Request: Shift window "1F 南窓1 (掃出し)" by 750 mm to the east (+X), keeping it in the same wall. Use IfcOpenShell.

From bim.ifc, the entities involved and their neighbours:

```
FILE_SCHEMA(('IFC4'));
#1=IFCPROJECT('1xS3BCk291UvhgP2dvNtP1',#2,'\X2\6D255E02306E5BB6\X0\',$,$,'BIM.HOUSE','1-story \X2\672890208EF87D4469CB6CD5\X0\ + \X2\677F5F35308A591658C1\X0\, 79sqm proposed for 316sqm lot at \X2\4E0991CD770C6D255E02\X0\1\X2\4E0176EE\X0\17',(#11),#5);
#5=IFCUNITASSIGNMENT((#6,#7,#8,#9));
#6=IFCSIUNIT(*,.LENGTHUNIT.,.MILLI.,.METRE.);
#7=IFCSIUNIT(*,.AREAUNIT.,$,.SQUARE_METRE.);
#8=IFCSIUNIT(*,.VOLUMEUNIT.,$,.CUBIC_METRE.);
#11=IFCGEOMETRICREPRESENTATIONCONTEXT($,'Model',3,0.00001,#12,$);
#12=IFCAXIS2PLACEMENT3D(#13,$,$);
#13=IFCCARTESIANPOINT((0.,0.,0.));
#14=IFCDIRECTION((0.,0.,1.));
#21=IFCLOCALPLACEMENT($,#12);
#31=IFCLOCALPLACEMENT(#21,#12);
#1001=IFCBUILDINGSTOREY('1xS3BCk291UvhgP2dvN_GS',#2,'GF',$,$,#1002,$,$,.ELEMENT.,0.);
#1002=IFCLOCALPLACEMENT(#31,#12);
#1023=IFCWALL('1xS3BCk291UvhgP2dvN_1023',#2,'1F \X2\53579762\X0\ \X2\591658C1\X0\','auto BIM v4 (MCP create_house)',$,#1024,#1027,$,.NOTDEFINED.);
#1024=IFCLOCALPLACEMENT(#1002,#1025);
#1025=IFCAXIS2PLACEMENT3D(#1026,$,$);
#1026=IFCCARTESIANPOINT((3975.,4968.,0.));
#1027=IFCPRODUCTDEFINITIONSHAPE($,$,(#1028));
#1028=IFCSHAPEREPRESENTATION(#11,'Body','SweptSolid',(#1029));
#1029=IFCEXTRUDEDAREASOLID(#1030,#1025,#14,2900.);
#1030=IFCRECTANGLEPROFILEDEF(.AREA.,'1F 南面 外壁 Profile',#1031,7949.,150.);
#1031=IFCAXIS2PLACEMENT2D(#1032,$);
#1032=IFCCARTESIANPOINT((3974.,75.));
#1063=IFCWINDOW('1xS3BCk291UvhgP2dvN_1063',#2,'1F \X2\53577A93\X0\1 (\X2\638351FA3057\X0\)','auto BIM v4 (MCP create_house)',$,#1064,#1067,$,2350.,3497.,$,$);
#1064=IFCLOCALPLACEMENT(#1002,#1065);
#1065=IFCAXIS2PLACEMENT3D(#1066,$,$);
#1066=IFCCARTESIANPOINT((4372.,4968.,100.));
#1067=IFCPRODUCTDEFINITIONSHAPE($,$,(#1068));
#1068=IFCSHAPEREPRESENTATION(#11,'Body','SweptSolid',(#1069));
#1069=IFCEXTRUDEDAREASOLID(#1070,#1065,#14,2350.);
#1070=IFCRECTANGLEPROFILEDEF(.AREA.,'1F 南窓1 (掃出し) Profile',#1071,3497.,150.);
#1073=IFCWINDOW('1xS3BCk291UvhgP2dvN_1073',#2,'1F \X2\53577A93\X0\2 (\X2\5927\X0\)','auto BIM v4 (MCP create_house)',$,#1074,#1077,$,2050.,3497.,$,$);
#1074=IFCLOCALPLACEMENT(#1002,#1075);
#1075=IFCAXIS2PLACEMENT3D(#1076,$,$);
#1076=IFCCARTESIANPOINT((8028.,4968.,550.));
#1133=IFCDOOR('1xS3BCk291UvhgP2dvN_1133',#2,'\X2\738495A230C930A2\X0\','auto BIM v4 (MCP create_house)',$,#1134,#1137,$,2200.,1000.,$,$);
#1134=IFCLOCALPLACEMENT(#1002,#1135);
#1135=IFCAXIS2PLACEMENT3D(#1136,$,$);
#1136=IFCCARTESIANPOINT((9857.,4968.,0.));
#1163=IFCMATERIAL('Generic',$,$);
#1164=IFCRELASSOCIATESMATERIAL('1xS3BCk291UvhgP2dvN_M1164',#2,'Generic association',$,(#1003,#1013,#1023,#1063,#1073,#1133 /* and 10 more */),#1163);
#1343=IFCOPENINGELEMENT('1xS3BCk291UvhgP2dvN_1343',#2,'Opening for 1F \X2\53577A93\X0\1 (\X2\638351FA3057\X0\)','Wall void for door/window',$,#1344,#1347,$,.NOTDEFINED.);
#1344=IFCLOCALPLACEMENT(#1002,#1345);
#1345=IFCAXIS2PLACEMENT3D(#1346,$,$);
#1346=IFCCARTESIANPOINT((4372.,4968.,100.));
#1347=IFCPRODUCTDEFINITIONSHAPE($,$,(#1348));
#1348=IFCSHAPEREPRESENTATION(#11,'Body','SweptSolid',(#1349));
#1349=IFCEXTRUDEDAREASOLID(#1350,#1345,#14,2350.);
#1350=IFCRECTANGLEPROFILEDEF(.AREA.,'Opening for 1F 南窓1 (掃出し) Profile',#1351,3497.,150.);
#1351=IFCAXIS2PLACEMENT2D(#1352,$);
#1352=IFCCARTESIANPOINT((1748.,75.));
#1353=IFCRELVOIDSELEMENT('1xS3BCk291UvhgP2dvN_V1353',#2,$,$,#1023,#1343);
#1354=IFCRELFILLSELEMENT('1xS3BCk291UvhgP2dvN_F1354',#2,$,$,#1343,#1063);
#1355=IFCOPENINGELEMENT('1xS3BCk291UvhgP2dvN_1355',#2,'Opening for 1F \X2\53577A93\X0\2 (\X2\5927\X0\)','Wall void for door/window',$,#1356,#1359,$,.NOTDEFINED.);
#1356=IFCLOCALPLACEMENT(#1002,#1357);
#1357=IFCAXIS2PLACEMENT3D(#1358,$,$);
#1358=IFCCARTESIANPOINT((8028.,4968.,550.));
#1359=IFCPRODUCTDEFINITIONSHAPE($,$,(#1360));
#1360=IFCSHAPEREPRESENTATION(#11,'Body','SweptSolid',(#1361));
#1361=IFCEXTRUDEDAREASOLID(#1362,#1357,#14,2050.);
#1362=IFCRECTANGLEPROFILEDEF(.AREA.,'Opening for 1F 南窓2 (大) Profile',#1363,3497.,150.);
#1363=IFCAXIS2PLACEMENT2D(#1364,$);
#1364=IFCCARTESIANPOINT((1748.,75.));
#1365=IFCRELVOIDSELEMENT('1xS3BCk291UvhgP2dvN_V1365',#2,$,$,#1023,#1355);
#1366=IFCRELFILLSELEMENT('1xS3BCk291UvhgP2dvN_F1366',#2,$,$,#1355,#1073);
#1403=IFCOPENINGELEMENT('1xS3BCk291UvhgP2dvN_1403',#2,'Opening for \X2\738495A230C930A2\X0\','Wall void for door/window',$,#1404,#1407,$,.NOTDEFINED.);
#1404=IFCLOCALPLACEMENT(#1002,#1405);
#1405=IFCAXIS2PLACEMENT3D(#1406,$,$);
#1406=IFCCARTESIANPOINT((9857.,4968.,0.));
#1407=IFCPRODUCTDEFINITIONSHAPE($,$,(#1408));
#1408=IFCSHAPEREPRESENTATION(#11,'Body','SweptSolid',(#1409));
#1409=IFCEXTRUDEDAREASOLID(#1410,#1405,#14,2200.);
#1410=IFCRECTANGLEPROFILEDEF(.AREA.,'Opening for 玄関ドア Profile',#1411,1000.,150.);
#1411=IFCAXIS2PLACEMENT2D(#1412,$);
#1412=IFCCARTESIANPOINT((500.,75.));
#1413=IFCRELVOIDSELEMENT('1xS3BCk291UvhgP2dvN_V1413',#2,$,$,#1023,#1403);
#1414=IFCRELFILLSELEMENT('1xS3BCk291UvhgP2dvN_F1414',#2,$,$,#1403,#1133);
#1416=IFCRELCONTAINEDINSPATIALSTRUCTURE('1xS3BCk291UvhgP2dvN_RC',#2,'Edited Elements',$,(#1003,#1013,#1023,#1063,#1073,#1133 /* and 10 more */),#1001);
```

```python
import ifcopenshell
import ifcopenshell.api.geometry
import ifcopenshell.util.placement
import ifcopenshell.util.unit

model = ifcopenshell.open("bim.ifc")
unit_scale = ifcopenshell.util.unit.calculate_unit_scale(model)

window = model.by_id(1063)
opening = window.FillsVoids[0].RelatingOpeningElement
wall = opening.VoidsElements[0].RelatingBuildingElement

wall_matrix = ifcopenshell.util.placement.get_local_placement(wall.ObjectPlacement)
shift = wall_matrix[:3, 0] * 0.75 / unit_scale
before = ifcopenshell.util.placement.get_local_placement(window.ObjectPlacement)[:3, 3].copy()

# The window is not placed relative to its opening, so move both.
for product in (opening, window):
    matrix = ifcopenshell.util.placement.get_local_placement(product.ObjectPlacement)
    matrix[:3, 3] += shift
    ifcopenshell.api.geometry.edit_object_placement(model, product=product, matrix=matrix, is_si=False)

after = ifcopenshell.util.placement.get_local_placement(window.ObjectPlacement)[:3, 3]
print("window moved by", (after - before).round(3) + 0.0)

model.write("bim_v2.ifc")
```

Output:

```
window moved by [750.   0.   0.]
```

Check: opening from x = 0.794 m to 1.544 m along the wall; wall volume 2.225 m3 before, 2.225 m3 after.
